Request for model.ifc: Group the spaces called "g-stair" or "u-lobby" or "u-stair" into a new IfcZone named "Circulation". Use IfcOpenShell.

First a look at what the model holds.

```python
import ifcopenshell

model = ifcopenshell.open("model.ifc")
print(model.schema)
seen = {}
for space in model.by_type("IfcSpace"):
    seen[space.LongName] = seen.get(space.LongName, 0) + 1
for name, count in sorted(seen.items(), key=str):
    print(count, "x", name)
print("zones:", [z.Name for z in model.by_type("IfcZone")][:20])
```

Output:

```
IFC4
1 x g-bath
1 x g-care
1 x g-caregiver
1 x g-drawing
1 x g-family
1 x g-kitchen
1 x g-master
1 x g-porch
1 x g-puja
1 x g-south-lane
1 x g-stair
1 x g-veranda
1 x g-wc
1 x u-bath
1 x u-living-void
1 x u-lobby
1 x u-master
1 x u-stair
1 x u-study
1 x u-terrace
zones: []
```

```python
import ifcopenshell
import ifcopenshell.api.group
import ifcopenshell.api.root

model = ifcopenshell.open("model.ifc")

names = {"g-stair", "u-lobby", "u-stair"}
spaces = [s for s in model.by_type("IfcSpace") if s.LongName in names]

zone = ifcopenshell.api.root.create_entity(model, ifc_class="IfcZone", name="Circulation")
ifcopenshell.api.group.assign_group(model, products=spaces, group=zone)
print(len(spaces), "spaces in", zone.Name)

model.write("model-out.ifc")
```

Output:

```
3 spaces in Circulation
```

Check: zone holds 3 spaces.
